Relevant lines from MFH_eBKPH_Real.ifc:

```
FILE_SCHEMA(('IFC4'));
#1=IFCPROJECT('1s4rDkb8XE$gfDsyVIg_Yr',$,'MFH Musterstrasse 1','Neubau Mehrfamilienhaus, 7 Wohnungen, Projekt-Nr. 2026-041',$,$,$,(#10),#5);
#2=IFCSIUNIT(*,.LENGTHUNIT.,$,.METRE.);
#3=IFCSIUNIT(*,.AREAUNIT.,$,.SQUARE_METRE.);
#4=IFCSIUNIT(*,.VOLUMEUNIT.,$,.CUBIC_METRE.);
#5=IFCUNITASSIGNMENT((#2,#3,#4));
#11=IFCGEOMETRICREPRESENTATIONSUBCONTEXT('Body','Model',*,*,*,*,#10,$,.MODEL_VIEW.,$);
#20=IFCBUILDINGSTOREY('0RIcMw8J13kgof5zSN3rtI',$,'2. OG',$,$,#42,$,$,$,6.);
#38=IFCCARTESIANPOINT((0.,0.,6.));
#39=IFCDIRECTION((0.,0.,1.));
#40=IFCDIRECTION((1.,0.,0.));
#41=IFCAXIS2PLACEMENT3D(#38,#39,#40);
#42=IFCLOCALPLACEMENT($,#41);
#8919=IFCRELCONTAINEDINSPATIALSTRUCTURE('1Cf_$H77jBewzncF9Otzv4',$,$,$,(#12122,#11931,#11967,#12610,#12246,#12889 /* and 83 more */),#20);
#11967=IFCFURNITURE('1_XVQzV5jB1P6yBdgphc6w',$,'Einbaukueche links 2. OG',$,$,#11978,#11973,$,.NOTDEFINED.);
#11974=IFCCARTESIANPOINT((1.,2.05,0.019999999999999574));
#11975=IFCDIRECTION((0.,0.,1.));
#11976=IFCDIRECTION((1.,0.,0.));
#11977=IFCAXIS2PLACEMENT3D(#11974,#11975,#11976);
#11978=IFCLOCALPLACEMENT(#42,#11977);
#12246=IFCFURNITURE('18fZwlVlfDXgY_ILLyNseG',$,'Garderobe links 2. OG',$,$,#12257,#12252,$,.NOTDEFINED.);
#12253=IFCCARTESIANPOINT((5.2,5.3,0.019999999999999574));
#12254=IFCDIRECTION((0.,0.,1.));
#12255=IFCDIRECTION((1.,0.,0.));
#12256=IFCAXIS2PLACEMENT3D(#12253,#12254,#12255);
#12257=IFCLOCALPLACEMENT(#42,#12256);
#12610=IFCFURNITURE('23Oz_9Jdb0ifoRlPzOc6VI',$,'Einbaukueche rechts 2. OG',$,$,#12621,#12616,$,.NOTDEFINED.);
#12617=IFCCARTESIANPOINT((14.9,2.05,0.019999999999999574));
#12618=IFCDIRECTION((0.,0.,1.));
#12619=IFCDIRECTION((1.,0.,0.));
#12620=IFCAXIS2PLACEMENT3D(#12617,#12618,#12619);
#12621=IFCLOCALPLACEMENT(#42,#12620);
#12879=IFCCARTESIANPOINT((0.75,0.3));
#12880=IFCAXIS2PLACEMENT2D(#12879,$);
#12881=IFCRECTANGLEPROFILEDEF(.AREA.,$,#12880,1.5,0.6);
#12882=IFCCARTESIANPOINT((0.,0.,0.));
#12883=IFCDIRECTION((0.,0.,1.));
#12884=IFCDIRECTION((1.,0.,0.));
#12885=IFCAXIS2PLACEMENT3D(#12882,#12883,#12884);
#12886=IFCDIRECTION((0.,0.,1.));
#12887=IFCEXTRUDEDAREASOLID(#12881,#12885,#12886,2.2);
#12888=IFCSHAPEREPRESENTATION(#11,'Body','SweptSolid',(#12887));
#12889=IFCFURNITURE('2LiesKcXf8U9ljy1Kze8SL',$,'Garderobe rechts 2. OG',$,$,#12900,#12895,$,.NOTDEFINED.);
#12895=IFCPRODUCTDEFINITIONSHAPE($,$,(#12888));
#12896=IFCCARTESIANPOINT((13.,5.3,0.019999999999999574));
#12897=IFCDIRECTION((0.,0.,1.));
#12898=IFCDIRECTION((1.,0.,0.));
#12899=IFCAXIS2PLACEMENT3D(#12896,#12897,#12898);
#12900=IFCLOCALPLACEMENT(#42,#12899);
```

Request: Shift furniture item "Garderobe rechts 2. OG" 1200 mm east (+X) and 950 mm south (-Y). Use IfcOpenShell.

```python
import ifcopenshell
import ifcopenshell.api.geometry
import ifcopenshell.util.placement
import ifcopenshell.util.unit

model = ifcopenshell.open("MFH_eBKPH_Real.ifc")
unit_scale = ifcopenshell.util.unit.calculate_unit_scale(model)

item = model.by_guid("2LiesKcXf8U9ljy1Kze8SL")
matrix = ifcopenshell.util.placement.get_local_placement(item.ObjectPlacement)
matrix[0, 3] += 1.2 / unit_scale
matrix[1, 3] -= 0.95 / unit_scale
ifcopenshell.api.geometry.edit_object_placement(model, product=item, matrix=matrix, is_si=False)

print(ifcopenshell.util.placement.get_local_placement(item.ObjectPlacement).round(3) + 0.0)

model.write("MFH_eBKPH_Real_edited.ifc")
```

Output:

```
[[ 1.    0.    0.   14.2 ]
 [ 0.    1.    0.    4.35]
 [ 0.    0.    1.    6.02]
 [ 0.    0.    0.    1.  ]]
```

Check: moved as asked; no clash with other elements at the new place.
